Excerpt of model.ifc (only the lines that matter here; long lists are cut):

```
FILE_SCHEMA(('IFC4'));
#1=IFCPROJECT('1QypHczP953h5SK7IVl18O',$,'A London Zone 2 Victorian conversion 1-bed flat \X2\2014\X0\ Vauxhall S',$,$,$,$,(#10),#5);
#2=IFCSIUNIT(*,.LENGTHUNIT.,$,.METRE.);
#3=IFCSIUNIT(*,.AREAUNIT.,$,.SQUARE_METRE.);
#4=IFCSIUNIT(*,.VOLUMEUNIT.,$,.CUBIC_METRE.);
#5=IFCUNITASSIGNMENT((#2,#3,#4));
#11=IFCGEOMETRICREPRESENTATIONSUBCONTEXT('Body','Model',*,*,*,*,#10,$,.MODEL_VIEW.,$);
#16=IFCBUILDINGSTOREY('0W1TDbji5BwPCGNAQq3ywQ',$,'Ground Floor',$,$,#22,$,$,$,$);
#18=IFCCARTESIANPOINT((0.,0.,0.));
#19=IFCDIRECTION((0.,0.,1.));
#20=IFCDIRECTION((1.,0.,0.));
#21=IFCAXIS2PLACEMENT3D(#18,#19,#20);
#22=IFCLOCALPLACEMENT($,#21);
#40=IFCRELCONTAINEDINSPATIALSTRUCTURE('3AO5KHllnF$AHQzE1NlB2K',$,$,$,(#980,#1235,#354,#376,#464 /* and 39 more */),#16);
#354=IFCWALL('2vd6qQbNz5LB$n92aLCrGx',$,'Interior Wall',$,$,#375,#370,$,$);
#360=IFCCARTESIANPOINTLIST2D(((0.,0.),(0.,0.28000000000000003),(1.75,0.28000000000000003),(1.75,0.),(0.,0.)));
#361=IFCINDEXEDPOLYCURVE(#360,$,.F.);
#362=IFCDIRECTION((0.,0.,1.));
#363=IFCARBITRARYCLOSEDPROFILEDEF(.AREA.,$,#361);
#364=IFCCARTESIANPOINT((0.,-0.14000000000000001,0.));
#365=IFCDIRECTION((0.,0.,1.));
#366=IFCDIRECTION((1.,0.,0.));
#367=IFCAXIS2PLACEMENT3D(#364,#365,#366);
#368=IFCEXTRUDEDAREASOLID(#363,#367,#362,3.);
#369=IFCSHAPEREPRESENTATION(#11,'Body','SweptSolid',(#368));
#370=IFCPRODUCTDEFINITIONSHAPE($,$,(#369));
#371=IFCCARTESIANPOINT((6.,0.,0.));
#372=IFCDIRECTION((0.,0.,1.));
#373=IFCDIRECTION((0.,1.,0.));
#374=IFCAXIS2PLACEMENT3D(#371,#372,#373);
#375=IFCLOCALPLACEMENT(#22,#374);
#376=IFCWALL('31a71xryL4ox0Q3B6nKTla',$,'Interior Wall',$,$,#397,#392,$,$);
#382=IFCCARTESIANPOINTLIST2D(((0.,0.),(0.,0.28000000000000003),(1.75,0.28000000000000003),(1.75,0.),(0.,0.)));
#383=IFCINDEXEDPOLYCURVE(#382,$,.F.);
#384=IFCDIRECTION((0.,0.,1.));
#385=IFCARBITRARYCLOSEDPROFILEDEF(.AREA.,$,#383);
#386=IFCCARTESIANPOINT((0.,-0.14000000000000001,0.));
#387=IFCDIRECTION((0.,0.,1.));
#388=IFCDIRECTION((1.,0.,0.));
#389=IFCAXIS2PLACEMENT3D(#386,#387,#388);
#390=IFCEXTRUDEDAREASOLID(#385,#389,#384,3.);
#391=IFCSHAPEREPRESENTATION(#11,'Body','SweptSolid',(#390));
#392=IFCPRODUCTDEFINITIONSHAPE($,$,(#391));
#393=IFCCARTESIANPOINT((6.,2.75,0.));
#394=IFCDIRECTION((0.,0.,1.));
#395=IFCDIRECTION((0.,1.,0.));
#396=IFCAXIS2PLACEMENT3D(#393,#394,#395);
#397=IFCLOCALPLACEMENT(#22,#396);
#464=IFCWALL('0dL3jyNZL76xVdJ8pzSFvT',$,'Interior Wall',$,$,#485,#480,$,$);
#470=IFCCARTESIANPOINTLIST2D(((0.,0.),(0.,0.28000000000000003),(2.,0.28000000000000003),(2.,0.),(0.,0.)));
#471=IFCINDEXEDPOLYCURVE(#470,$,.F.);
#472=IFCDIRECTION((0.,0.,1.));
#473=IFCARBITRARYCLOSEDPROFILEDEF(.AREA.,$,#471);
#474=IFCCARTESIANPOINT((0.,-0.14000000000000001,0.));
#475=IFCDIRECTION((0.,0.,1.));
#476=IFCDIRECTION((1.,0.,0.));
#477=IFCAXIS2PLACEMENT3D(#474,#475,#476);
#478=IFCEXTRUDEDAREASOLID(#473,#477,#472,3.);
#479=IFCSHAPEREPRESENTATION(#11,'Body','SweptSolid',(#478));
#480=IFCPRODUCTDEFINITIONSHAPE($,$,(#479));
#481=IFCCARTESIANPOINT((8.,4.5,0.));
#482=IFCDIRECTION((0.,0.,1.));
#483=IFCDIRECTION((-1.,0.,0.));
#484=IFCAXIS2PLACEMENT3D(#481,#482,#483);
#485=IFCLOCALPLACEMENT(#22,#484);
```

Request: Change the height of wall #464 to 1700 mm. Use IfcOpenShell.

```python
import ifcopenshell
import ifcopenshell.geom
import ifcopenshell.util.representation
import ifcopenshell.util.shape
import ifcopenshell.util.unit

model = ifcopenshell.open("model.ifc")
unit_scale = ifcopenshell.util.unit.calculate_unit_scale(model)
settings = ifcopenshell.geom.settings()


def volume(element):
    """Net volume in cubic metres, openings subtracted."""
    shape = ifcopenshell.geom.create_shape(settings, element)
    return ifcopenshell.util.shape.get_volume(shape.geometry)


wall = model.by_id(464)
before = volume(wall)

body = ifcopenshell.util.representation.get_representation(wall, "Model", "Body")
solid = body.Items[0]
old_height = solid.Depth
solid.Depth = 1.7 / unit_scale
after = volume(wall)

print(f"height {old_height:g} -> {solid.Depth:g}, volume {before:.3f} -> {after:.3f} m3")

model.write("model_v2.ifc")
```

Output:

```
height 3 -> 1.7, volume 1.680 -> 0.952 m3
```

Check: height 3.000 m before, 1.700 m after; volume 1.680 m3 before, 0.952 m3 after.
